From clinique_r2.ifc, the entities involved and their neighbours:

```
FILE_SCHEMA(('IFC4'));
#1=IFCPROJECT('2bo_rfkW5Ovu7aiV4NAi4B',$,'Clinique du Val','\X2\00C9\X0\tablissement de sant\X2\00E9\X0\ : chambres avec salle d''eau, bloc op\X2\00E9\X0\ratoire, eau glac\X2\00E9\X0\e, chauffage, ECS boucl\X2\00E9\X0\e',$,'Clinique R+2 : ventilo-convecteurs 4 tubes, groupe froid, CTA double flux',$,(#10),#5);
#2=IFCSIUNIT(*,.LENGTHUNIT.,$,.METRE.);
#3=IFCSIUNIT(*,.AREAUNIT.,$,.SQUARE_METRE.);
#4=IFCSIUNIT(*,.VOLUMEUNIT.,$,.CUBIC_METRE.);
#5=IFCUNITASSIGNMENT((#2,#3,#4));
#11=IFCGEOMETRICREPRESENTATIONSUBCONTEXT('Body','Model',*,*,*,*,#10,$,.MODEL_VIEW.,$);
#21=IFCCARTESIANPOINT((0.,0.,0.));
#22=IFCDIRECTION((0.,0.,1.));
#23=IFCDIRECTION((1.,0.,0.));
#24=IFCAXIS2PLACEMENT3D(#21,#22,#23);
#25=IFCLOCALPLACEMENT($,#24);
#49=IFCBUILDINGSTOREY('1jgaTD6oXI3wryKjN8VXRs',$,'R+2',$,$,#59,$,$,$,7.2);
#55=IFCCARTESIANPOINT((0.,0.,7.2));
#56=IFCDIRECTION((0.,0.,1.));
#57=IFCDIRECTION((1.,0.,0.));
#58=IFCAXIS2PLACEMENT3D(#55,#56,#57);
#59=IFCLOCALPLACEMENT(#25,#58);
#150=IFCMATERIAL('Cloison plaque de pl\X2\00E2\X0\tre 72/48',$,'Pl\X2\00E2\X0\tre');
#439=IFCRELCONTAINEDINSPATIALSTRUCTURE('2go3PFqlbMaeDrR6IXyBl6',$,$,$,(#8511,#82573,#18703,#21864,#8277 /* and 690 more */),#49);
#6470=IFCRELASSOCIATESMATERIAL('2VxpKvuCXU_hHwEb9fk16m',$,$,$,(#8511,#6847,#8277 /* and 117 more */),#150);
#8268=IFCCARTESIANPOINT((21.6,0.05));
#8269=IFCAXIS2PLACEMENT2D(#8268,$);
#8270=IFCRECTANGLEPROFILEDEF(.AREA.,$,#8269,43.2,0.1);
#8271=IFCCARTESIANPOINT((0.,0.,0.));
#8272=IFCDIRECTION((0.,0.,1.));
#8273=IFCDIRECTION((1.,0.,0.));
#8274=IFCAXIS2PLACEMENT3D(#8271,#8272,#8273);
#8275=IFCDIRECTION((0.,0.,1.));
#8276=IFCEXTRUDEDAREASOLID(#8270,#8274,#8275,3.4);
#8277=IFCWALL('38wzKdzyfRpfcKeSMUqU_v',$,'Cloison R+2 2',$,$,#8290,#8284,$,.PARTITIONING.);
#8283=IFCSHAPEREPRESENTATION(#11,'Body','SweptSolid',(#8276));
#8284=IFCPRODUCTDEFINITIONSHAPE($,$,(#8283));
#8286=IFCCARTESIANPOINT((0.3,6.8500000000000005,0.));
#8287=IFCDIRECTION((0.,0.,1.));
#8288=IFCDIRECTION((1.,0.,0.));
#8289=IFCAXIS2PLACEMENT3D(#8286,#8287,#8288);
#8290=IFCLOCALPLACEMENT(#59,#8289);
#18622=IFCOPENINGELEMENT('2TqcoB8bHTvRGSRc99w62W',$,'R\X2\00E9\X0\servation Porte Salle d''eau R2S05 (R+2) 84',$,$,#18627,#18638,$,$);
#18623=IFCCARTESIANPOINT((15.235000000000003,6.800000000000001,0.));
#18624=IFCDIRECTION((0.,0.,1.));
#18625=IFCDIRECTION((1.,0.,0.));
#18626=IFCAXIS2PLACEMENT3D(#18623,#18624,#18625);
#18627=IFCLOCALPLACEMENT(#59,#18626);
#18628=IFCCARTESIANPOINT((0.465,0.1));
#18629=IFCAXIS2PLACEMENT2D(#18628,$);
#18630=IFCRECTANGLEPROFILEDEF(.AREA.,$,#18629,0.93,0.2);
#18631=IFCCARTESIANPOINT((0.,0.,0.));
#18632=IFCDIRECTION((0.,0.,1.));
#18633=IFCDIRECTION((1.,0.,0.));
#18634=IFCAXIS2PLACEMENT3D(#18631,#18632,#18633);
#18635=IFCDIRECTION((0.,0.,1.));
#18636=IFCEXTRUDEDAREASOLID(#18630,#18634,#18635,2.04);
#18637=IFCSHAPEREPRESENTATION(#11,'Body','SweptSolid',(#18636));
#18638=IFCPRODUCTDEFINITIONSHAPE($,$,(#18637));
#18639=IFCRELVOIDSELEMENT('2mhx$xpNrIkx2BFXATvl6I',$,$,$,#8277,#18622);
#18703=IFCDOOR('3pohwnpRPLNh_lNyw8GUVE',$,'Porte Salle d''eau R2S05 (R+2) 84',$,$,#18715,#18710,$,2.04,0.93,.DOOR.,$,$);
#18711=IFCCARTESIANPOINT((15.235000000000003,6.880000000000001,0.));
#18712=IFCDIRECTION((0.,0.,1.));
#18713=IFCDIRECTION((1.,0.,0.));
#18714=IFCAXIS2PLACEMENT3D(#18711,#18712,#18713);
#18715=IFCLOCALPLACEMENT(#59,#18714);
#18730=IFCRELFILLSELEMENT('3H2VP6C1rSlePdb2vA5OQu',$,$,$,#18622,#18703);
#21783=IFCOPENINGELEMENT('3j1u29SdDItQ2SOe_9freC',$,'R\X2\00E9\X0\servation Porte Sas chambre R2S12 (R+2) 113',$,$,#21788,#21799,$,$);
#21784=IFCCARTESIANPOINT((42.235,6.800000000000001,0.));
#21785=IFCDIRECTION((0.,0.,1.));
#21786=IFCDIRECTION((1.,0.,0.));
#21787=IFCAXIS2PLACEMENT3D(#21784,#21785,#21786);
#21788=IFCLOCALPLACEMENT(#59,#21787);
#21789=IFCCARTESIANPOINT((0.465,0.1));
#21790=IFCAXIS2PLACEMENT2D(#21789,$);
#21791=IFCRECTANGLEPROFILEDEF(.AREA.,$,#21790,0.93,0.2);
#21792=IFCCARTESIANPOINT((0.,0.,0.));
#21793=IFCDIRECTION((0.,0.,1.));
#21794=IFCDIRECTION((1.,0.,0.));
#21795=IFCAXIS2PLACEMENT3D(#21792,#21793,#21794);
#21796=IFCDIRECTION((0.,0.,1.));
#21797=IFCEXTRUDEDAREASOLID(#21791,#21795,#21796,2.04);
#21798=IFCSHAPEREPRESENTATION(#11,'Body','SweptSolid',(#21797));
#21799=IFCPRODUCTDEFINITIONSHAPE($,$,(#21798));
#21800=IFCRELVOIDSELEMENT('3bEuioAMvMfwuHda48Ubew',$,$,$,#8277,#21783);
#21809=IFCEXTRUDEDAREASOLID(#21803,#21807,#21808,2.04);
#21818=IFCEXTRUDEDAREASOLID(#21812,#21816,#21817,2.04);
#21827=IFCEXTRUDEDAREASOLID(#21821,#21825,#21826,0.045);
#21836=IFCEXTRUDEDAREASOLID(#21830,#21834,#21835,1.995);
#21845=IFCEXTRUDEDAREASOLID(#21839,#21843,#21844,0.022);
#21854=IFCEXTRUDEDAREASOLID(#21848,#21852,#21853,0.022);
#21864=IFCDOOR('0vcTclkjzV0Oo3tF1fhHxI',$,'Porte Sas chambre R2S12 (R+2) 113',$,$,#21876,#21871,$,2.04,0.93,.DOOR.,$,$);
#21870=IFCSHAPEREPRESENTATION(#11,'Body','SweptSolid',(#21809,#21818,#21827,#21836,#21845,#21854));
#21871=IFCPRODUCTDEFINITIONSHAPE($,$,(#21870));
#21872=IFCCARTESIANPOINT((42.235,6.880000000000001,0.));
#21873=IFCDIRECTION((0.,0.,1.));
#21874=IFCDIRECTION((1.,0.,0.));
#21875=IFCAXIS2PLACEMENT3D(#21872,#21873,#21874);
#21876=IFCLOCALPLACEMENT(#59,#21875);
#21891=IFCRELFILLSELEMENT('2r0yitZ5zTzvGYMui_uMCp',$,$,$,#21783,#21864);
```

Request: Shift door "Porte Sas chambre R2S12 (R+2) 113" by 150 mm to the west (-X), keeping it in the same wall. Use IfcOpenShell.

```python
import ifcopenshell
import ifcopenshell.api.geometry
import ifcopenshell.util.placement

model = ifcopenshell.open("clinique_r2.ifc")

door = model.by_guid("0vcTclkjzV0Oo3tF1fhHxI")
opening = door.FillsVoids[0].RelatingOpeningElement
wall = opening.VoidsElements[0].RelatingBuildingElement

wall_matrix = ifcopenshell.util.placement.get_local_placement(wall.ObjectPlacement)
shift = wall_matrix[:3, 0] * -0.15
before = ifcopenshell.util.placement.get_local_placement(door.ObjectPlacement)[:3, 3].copy()

# The door is not placed relative to its opening, so move both.
for product in (opening, door):
    matrix = ifcopenshell.util.placement.get_local_placement(product.ObjectPlacement)
    matrix[:3, 3] += shift
    ifcopenshell.api.geometry.edit_object_placement(model, product=product, matrix=matrix, is_si=False)

after = ifcopenshell.util.placement.get_local_placement(door.ObjectPlacement)[:3, 3]
print("door moved by", (after - before).round(3) + 0.0)

model.write("clinique_r2_v2.ifc")
```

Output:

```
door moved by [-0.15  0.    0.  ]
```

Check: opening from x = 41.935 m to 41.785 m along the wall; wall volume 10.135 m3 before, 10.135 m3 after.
